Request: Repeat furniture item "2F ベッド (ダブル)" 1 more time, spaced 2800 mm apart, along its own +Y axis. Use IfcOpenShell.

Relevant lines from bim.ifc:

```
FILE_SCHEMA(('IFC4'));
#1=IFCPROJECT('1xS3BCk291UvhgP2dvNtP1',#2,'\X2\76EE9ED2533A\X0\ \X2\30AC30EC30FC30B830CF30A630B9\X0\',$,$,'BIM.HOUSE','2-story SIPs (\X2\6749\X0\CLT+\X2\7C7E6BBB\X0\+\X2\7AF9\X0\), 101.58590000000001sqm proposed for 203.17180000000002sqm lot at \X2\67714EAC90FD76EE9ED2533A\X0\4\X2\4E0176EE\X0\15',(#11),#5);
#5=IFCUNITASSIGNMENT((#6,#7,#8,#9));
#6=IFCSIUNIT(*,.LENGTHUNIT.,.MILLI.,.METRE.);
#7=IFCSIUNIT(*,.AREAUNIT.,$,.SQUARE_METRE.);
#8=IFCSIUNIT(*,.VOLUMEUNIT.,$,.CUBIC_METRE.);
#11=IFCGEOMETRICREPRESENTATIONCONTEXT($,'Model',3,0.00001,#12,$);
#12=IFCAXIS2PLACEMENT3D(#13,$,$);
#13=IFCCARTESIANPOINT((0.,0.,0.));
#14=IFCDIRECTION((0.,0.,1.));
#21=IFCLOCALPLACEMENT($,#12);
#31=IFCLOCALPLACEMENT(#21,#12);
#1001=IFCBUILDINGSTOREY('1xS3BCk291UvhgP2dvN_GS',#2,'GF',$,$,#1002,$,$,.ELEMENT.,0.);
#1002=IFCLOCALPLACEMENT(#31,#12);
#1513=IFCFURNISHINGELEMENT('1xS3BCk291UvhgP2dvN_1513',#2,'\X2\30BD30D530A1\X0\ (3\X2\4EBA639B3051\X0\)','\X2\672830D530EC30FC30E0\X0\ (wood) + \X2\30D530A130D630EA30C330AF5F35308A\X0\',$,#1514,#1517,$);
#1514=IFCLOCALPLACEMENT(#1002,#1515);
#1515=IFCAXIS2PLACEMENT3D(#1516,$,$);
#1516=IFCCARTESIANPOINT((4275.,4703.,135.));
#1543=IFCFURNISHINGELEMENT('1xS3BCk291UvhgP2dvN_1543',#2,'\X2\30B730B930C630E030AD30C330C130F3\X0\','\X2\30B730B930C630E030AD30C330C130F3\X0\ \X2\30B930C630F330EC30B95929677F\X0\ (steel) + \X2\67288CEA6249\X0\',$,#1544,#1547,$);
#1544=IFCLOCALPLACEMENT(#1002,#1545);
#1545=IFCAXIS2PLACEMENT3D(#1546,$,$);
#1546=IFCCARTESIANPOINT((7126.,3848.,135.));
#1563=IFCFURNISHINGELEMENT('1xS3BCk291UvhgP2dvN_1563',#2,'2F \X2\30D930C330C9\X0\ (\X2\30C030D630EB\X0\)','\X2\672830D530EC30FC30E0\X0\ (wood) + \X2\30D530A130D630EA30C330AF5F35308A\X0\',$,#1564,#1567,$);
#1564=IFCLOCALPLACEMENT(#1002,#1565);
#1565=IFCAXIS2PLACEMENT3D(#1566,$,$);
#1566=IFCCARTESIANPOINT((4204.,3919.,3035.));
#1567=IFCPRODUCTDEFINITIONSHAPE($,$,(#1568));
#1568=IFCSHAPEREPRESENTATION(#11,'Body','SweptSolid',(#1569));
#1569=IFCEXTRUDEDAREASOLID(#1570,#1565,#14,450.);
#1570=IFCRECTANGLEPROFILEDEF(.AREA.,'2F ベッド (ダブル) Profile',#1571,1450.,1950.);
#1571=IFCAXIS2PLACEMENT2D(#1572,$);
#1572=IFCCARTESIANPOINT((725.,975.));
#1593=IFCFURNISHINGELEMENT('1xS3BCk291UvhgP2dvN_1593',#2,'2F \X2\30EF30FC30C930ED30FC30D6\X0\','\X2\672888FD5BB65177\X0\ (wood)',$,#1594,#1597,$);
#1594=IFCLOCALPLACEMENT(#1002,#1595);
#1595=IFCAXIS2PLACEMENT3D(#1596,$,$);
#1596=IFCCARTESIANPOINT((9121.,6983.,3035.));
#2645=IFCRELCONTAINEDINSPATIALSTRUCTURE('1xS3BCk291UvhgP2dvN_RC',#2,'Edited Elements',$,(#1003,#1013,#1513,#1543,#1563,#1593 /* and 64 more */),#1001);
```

```python
import ifcopenshell
import ifcopenshell.api.geometry
import ifcopenshell.api.root
import ifcopenshell.util.element
import ifcopenshell.util.placement

model = ifcopenshell.open("bim.ifc")


def reuse_history(source, copy):
    """copy_class also copies each property set's owner history, people and application; keep the originals."""
    for rel in copy.IsDefinedBy:
        if rel.is_a("IfcRelDefinesByProperties") and (history := rel.RelatingPropertyDefinition.OwnerHistory):
            rel.RelatingPropertyDefinition.OwnerHistory = source.OwnerHistory
            ifcopenshell.util.element.remove_deep2(model, history)


source = model.by_id(1563)
base = ifcopenshell.util.placement.get_local_placement(source.ObjectPlacement)
step = base[:3, 1] * 2800.0

for i in range(1, 2):
    copy = ifcopenshell.api.root.copy_class(model, product=source)
    copy.Representation = ifcopenshell.util.element.copy_deep(
        model, source.Representation, exclude=["IfcGeometricRepresentationContext", "IfcRepresentationMap"]
    )
    reuse_history(source, copy)
    matrix = base.copy()
    matrix[:3, 3] += i * step
    print("added at", matrix[:3, 3].round(3) + 0.0)
    ifcopenshell.api.geometry.edit_object_placement(model, product=copy, matrix=matrix, is_si=False)

model.write("bim_updated.ifc")
```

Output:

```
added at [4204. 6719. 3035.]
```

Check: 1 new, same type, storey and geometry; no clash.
